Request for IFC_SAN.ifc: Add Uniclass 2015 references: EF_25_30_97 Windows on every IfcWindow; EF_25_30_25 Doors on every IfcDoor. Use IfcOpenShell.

First a look at what the model holds.

```python
import ifcopenshell

model = ifcopenshell.open("IFC_SAN.ifc")
print(model.schema)
print("classifications:", [c.Name for c in model.by_type("IfcClassification")])
for ifc_class in ("IfcDoor", "IfcRoof", "IfcStair", "IfcWall", "IfcWindow"):
    print(ifc_class, len(model.by_type(ifc_class)))
```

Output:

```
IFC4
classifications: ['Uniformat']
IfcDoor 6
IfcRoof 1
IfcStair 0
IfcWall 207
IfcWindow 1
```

```python
import ifcopenshell
import ifcopenshell.api.classification

model = ifcopenshell.open("IFC_SAN.ifc")

system = ifcopenshell.api.classification.add_classification(model, classification="Uniclass 2015")

codes = {
    "IfcWindow": ("EF_25_30_97", "Windows"),
    "IfcDoor": ("EF_25_30_25", "Doors"),
}
for ifc_class, (code, name) in codes.items():
    products = model.by_type(ifc_class)
    ifcopenshell.api.classification.add_reference(
        model, products=products, classification=system, identification=code, name=name
    )
    print(code, len(products))

model.write("IFC_SAN_updated.ifc")
```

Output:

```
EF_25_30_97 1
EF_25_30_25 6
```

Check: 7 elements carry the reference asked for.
